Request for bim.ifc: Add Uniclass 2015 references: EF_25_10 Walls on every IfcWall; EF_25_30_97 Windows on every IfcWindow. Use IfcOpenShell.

First a look at what the model holds.

```python
import ifcopenshell

model = ifcopenshell.open("bim.ifc")
print(model.schema)
print("classifications:", [c.Name for c in model.by_type("IfcClassification")])
for ifc_class in ("IfcDoor", "IfcRoof", "IfcStair", "IfcWall", "IfcWindow"):
    print(ifc_class, len(model.by_type(ifc_class)))
```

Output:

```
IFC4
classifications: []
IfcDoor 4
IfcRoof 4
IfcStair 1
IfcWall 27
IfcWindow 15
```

```python
import ifcopenshell
import ifcopenshell.api.classification

model = ifcopenshell.open("bim.ifc")

system = ifcopenshell.api.classification.add_classification(model, classification="Uniclass 2015")

codes = {
    "IfcWall": ("EF_25_10", "Walls"),
    "IfcWindow": ("EF_25_30_97", "Windows"),
}
for ifc_class, (code, name) in codes.items():
    products = model.by_type(ifc_class)
    ifcopenshell.api.classification.add_reference(
        model, products=products, classification=system, identification=code, name=name
    )
    print(code, len(products))

model.write("bim_edited.ifc")
```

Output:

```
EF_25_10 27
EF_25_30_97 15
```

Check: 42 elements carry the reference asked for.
